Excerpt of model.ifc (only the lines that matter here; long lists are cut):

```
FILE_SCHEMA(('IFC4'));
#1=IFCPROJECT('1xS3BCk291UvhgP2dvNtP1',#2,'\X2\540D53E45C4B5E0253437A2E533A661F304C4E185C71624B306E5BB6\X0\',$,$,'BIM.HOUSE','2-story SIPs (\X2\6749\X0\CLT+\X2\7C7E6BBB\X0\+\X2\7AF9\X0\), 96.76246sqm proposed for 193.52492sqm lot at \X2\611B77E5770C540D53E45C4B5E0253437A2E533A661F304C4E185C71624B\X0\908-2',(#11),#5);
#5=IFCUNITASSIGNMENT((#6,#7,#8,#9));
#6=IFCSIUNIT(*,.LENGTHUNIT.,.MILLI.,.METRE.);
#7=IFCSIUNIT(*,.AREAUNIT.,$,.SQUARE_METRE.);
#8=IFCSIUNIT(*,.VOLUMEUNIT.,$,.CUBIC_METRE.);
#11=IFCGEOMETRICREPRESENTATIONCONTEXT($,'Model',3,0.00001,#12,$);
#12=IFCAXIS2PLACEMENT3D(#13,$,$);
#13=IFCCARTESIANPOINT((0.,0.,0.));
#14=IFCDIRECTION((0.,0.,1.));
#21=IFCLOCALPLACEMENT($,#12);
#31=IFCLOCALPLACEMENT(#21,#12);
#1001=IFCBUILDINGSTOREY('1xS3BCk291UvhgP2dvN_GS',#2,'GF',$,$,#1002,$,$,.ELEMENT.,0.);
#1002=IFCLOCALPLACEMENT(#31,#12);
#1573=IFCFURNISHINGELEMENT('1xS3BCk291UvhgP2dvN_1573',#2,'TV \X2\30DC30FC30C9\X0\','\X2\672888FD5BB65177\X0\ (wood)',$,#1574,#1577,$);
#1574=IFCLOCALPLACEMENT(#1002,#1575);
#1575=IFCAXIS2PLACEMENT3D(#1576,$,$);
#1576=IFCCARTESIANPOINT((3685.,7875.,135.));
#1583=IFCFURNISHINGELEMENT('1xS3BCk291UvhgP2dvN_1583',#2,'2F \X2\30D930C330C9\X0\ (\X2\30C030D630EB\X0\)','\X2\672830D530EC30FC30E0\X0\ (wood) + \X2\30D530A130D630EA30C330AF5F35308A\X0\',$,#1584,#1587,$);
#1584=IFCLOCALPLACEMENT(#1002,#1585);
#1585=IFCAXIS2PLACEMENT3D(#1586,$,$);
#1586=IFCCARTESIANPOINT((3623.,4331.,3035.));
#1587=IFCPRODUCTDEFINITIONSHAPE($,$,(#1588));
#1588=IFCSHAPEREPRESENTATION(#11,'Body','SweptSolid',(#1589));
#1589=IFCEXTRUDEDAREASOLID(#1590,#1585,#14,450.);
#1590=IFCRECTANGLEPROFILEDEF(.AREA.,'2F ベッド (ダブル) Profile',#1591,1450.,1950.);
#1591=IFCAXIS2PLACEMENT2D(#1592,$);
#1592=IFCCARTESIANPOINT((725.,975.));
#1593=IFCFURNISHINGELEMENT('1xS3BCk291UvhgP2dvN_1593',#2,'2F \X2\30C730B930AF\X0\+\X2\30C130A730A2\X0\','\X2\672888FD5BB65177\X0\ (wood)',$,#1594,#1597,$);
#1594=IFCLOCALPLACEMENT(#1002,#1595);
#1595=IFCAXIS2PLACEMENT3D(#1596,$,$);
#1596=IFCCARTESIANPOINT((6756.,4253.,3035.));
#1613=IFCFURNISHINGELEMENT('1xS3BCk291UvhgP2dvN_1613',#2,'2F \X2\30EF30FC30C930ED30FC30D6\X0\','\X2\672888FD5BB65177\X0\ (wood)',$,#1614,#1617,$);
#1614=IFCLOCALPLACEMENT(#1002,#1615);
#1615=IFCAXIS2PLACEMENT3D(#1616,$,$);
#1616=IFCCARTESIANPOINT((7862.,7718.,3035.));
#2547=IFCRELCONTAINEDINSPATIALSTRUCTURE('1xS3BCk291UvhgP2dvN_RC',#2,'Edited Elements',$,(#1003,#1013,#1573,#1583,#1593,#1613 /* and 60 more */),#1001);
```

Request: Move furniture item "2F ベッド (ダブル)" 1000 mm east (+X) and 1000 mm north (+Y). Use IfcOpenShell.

```python
import ifcopenshell
import ifcopenshell.api.geometry
import ifcopenshell.util.placement
import ifcopenshell.util.unit

model = ifcopenshell.open("model.ifc")
unit_scale = ifcopenshell.util.unit.calculate_unit_scale(model)

item = model.by_id(1583)
matrix = ifcopenshell.util.placement.get_local_placement(item.ObjectPlacement)
matrix[0, 3] += 1 / unit_scale
matrix[1, 3] += 1 / unit_scale
ifcopenshell.api.geometry.edit_object_placement(model, product=item, matrix=matrix, is_si=False)

print(ifcopenshell.util.placement.get_local_placement(item.ObjectPlacement).round(3) + 0.0)

model.write("model_edited.ifc")
```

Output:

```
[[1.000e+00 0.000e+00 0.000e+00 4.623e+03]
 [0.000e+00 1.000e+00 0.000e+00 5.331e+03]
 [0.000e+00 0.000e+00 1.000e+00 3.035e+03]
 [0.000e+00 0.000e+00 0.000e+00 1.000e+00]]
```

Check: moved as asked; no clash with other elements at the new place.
